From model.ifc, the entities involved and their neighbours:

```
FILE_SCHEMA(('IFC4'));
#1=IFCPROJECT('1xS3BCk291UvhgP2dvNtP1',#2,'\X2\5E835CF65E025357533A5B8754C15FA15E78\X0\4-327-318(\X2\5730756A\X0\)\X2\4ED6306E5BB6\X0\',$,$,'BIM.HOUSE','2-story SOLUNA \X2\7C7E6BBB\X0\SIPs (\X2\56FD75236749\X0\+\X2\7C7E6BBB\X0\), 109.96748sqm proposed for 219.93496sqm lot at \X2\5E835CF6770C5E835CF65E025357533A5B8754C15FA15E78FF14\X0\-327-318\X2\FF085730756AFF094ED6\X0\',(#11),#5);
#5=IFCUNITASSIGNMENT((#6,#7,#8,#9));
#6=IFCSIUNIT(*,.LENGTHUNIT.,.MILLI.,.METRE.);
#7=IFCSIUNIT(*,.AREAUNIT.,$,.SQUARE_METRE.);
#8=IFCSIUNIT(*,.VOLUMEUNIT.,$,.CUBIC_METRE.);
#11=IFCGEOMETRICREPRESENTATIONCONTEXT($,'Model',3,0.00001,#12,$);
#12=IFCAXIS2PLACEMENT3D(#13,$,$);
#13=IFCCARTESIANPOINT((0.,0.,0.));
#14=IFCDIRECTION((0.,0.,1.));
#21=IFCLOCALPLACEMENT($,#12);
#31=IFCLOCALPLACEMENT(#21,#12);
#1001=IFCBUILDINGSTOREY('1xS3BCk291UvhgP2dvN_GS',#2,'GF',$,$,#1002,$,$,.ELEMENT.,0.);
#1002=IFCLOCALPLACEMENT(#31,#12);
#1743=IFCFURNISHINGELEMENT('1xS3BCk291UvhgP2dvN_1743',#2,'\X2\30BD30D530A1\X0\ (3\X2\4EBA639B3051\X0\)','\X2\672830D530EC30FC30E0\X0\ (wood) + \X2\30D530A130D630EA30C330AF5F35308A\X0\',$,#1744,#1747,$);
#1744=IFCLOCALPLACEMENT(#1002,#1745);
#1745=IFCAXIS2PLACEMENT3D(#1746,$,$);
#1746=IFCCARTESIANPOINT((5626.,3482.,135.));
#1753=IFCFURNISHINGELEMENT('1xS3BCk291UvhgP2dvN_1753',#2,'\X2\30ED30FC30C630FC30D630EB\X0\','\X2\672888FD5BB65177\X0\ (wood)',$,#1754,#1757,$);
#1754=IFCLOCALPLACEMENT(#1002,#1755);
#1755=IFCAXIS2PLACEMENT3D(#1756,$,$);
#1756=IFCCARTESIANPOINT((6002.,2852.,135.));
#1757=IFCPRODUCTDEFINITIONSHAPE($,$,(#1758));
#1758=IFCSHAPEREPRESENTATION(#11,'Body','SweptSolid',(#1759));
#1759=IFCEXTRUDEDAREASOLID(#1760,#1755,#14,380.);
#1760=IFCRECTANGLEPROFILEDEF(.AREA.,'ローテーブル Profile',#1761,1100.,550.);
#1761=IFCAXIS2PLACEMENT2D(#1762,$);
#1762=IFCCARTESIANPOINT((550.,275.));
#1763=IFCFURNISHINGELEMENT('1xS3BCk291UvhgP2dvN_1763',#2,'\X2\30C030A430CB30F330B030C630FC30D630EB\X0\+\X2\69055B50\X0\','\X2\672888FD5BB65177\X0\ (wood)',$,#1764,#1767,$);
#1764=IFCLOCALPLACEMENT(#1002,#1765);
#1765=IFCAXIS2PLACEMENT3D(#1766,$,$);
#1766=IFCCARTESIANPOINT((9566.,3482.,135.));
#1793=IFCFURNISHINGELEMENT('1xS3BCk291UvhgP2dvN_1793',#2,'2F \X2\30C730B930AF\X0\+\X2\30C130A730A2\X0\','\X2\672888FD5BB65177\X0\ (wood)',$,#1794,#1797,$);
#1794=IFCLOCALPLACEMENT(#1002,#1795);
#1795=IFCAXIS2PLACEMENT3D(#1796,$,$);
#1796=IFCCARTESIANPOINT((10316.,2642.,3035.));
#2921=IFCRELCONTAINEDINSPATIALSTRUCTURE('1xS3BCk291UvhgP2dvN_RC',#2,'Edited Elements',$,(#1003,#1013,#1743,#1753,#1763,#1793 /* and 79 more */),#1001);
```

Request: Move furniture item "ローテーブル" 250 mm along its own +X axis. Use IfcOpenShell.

```python
import ifcopenshell
import ifcopenshell.api.geometry
import ifcopenshell.util.placement
import ifcopenshell.util.unit

model = ifcopenshell.open("model.ifc")
unit_scale = ifcopenshell.util.unit.calculate_unit_scale(model)

item = model.by_guid("1xS3BCk291UvhgP2dvN_1753")
matrix = ifcopenshell.util.placement.get_local_placement(item.ObjectPlacement)
matrix[:3, 3] += matrix[:3, 0] * 0.25 / unit_scale
ifcopenshell.api.geometry.edit_object_placement(model, product=item, matrix=matrix, is_si=False)

print(ifcopenshell.util.placement.get_local_placement(item.ObjectPlacement).round(3) + 0.0)

model.write("model_updated.ifc")
```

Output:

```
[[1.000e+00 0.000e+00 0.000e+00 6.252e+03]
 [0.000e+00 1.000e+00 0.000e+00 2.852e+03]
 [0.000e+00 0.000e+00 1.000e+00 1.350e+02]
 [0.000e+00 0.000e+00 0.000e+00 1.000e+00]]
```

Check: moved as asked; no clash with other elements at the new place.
